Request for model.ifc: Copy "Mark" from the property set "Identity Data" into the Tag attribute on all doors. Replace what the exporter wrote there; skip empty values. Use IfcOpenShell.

First a look at what the model holds.

```python
import ifcopenshell
import ifcopenshell.util.element

model = ifcopenshell.open("model.ifc")
print(model.schema)
doors = model.by_type("IfcDoor")
print(len(doors), "doors")
for e in doors[:8]:
    source = ifcopenshell.util.element.get_pset(e, "Identity Data", "Mark")
    target = e.Tag
    print(e.id(), repr(source), repr(target), sep=" | ")
```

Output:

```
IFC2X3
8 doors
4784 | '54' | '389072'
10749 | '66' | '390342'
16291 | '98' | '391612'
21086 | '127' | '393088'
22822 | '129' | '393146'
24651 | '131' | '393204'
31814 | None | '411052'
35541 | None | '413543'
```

```python
import ifcopenshell
import ifcopenshell.util.element

model = ifcopenshell.open("model.ifc")

count = 0
for e in model.by_type("IfcDoor"):
    value = ifcopenshell.util.element.get_pset(e, "Identity Data", "Mark")
    current = e.Tag
    if not value or not value.strip() or current == value:
        continue
    e.Tag = value
    count += 1

print(count, "doors updated")

model.write("model_edited.ifc")
```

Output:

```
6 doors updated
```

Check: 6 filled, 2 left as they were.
